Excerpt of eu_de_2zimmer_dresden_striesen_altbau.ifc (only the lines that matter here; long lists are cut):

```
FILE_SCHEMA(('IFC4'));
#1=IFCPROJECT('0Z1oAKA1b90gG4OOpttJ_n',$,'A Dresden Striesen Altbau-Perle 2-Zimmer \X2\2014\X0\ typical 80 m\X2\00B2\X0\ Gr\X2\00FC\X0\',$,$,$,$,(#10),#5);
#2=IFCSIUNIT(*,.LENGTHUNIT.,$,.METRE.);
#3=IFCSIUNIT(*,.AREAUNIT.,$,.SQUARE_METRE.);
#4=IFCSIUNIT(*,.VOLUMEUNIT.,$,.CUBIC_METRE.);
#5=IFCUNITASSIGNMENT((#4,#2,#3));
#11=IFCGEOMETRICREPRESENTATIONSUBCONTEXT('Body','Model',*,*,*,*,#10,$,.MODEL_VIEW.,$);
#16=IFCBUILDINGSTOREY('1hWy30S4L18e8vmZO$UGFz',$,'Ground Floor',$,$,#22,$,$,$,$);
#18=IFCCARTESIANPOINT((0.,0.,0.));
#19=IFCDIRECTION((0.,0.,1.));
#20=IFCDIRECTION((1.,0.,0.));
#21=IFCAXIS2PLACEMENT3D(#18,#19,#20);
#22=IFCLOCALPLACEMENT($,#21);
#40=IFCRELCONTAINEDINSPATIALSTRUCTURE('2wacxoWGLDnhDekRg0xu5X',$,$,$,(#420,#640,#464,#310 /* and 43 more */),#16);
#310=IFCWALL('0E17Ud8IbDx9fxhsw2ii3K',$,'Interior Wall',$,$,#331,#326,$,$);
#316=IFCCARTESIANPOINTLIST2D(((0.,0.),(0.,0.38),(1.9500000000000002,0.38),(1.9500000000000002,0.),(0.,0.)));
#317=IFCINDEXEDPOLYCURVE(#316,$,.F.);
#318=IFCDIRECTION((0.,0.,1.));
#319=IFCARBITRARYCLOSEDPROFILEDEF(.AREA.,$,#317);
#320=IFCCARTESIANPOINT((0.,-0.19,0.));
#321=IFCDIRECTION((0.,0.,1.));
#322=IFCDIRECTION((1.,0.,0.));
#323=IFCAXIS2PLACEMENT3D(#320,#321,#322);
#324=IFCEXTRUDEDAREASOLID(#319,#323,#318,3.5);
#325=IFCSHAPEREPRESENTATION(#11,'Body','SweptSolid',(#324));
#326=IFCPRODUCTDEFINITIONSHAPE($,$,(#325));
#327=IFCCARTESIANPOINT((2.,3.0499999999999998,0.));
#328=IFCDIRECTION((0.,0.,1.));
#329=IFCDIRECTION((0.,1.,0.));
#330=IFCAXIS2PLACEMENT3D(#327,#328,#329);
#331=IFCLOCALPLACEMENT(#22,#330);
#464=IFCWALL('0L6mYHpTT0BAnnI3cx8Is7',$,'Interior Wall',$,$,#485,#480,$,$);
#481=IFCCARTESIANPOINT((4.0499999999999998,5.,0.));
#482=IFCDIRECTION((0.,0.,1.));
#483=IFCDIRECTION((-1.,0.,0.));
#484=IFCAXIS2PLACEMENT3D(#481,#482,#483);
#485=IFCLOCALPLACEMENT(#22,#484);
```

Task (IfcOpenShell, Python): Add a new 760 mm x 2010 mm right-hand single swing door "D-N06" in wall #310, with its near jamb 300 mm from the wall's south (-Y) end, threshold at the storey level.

```python
import numpy as np
import ifcopenshell
import ifcopenshell.api.feature
import ifcopenshell.api.geometry
import ifcopenshell.api.root
import ifcopenshell.api.spatial
import ifcopenshell.geom
import ifcopenshell.util.element
import ifcopenshell.util.placement
import ifcopenshell.util.representation
import ifcopenshell.util.shape
import ifcopenshell.util.unit

model = ifcopenshell.open("eu_de_2zimmer_dresden_striesen_altbau.ifc")
unit_scale = ifcopenshell.util.unit.calculate_unit_scale(model)
settings = ifcopenshell.geom.settings()


def volume(element):
    """Net volume in cubic metres, openings subtracted."""
    shape = ifcopenshell.geom.create_shape(settings, element)
    return ifcopenshell.util.shape.get_volume(shape.geometry)


wall = model.by_guid("0E17Ud8IbDx9fxhsw2ii3K")
storey = ifcopenshell.util.element.get_container(wall, ifc_class="IfcBuildingStorey")
context = ifcopenshell.util.representation.get_context(model, "Model", "Body", "MODEL_VIEW")
before = volume(wall)

width, height, from_end, sill = 0.76, 2.01, 0.3, 0.0  # metres

# The wall runs along its own X axis, and the end named is its -X end.
wall_shape = ifcopenshell.geom.create_shape(settings, wall)
x, y, z = ifcopenshell.util.shape.get_vertices(wall_shape.geometry).T
start = x.min() + from_end
face, thickness = float(y.min()), float(y.max() - y.min())
wall_matrix = ifcopenshell.util.placement.get_local_placement(wall.ObjectPlacement)
level = ifcopenshell.util.placement.get_local_placement(storey.ObjectPlacement)[2, 3]


def in_wall(x, y):
    """Placement at x, y metres in the wall's axes, at sill height."""
    matrix = wall_matrix.copy()
    matrix[:, 3] = wall_matrix @ np.array([x / unit_scale, y / unit_scale, 0.0, 1.0])
    matrix[2, 3] = level + sill / unit_scale
    return matrix


# Opening: a box that overshoots both wall faces by 50 mm.
opening = ifcopenshell.api.root.create_entity(model, ifc_class="IfcOpeningElement", predefined_type="OPENING")
box = ifcopenshell.api.geometry.add_wall_representation(
    model, context=context, length=width, height=height, thickness=thickness + 0.1
)
ifcopenshell.api.geometry.assign_representation(model, product=opening, representation=box)
ifcopenshell.api.geometry.edit_object_placement(model, product=opening, matrix=in_wall(start, face - 0.05), is_si=False)
ifcopenshell.api.feature.add_feature(model, feature=opening, element=wall)

door = ifcopenshell.api.root.create_entity(model, ifc_class="IfcDoor", name="D-N06", predefined_type="DOOR")
door.OverallWidth, door.OverallHeight = width / unit_scale, height / unit_scale
door.OperationType = "SINGLE_SWING_RIGHT"
body = ifcopenshell.api.geometry.add_door_representation(
    model,
    context=context,
    overall_width=door.OverallWidth,
    overall_height=door.OverallHeight,
    operation_type="SINGLE_SWING_RIGHT",
    lining_properties={"LiningDepth": thickness / unit_scale, "ThresholdDepth": thickness / unit_scale},
)
ifcopenshell.api.geometry.assign_representation(model, product=door, representation=body)
ifcopenshell.api.spatial.assign_container(model, products=[door], relating_structure=storey)
ifcopenshell.api.feature.add_filling(model, opening=opening, element=door)

# The lining spans the wall, so the door starts at the wall face.
ifcopenshell.api.geometry.edit_object_placement(model, product=door, matrix=in_wall(start, face), is_si=False)

after = volume(wall)

print(f"wall volume {before:.3f} -> {after:.3f} m3")

model.write("eu_de_2zimmer_dresden_striesen_altbau_updated.ifc")
```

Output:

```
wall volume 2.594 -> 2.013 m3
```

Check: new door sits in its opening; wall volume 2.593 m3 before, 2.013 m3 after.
